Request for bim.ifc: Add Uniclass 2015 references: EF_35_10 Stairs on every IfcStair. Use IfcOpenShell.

First a look at what the model holds.

```python
import ifcopenshell

model = ifcopenshell.open("bim.ifc")
print(model.schema)
print("classifications:", [c.Name for c in model.by_type("IfcClassification")])
for ifc_class in ("IfcDoor", "IfcRoof", "IfcStair", "IfcWall", "IfcWindow"):
    print(ifc_class, len(model.by_type(ifc_class)))
```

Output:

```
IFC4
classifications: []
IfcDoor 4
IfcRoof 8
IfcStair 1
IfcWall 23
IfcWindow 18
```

```python
import ifcopenshell
import ifcopenshell.api.classification

model = ifcopenshell.open("bim.ifc")

system = ifcopenshell.api.classification.add_classification(model, classification="Uniclass 2015")

codes = {
    "IfcStair": ("EF_35_10", "Stairs"),
}
for ifc_class, (code, name) in codes.items():
    products = model.by_type(ifc_class)
    ifcopenshell.api.classification.add_reference(
        model, products=products, classification=system, identification=code, name=name
    )
    print(code, len(products))

model.write("bim-out.ifc")
```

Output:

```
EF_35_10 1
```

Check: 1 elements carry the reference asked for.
